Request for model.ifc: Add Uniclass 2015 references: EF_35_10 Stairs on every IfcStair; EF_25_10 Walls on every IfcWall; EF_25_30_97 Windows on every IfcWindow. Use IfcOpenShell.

First a look at what the model holds.

```python
import ifcopenshell

model = ifcopenshell.open("model.ifc")
print(model.schema)
print("classifications:", [c.Name for c in model.by_type("IfcClassification")])
for ifc_class in ("IfcDoor", "IfcRoof", "IfcStair", "IfcWall", "IfcWindow"):
    print(ifc_class, len(model.by_type(ifc_class)))
```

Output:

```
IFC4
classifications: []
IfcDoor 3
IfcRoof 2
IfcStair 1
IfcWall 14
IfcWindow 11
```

```python
import ifcopenshell
import ifcopenshell.api.classification

model = ifcopenshell.open("model.ifc")

system = ifcopenshell.api.classification.add_classification(model, classification="Uniclass 2015")

codes = {
    "IfcStair": ("EF_35_10", "Stairs"),
    "IfcWall": ("EF_25_10", "Walls"),
    "IfcWindow": ("EF_25_30_97", "Windows"),
}
for ifc_class, (code, name) in codes.items():
    products = model.by_type(ifc_class)
    ifcopenshell.api.classification.add_reference(
        model, products=products, classification=system, identification=code, name=name
    )
    print(code, len(products))

model.write("model-out.ifc")
```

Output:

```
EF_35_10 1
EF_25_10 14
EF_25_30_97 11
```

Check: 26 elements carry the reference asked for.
